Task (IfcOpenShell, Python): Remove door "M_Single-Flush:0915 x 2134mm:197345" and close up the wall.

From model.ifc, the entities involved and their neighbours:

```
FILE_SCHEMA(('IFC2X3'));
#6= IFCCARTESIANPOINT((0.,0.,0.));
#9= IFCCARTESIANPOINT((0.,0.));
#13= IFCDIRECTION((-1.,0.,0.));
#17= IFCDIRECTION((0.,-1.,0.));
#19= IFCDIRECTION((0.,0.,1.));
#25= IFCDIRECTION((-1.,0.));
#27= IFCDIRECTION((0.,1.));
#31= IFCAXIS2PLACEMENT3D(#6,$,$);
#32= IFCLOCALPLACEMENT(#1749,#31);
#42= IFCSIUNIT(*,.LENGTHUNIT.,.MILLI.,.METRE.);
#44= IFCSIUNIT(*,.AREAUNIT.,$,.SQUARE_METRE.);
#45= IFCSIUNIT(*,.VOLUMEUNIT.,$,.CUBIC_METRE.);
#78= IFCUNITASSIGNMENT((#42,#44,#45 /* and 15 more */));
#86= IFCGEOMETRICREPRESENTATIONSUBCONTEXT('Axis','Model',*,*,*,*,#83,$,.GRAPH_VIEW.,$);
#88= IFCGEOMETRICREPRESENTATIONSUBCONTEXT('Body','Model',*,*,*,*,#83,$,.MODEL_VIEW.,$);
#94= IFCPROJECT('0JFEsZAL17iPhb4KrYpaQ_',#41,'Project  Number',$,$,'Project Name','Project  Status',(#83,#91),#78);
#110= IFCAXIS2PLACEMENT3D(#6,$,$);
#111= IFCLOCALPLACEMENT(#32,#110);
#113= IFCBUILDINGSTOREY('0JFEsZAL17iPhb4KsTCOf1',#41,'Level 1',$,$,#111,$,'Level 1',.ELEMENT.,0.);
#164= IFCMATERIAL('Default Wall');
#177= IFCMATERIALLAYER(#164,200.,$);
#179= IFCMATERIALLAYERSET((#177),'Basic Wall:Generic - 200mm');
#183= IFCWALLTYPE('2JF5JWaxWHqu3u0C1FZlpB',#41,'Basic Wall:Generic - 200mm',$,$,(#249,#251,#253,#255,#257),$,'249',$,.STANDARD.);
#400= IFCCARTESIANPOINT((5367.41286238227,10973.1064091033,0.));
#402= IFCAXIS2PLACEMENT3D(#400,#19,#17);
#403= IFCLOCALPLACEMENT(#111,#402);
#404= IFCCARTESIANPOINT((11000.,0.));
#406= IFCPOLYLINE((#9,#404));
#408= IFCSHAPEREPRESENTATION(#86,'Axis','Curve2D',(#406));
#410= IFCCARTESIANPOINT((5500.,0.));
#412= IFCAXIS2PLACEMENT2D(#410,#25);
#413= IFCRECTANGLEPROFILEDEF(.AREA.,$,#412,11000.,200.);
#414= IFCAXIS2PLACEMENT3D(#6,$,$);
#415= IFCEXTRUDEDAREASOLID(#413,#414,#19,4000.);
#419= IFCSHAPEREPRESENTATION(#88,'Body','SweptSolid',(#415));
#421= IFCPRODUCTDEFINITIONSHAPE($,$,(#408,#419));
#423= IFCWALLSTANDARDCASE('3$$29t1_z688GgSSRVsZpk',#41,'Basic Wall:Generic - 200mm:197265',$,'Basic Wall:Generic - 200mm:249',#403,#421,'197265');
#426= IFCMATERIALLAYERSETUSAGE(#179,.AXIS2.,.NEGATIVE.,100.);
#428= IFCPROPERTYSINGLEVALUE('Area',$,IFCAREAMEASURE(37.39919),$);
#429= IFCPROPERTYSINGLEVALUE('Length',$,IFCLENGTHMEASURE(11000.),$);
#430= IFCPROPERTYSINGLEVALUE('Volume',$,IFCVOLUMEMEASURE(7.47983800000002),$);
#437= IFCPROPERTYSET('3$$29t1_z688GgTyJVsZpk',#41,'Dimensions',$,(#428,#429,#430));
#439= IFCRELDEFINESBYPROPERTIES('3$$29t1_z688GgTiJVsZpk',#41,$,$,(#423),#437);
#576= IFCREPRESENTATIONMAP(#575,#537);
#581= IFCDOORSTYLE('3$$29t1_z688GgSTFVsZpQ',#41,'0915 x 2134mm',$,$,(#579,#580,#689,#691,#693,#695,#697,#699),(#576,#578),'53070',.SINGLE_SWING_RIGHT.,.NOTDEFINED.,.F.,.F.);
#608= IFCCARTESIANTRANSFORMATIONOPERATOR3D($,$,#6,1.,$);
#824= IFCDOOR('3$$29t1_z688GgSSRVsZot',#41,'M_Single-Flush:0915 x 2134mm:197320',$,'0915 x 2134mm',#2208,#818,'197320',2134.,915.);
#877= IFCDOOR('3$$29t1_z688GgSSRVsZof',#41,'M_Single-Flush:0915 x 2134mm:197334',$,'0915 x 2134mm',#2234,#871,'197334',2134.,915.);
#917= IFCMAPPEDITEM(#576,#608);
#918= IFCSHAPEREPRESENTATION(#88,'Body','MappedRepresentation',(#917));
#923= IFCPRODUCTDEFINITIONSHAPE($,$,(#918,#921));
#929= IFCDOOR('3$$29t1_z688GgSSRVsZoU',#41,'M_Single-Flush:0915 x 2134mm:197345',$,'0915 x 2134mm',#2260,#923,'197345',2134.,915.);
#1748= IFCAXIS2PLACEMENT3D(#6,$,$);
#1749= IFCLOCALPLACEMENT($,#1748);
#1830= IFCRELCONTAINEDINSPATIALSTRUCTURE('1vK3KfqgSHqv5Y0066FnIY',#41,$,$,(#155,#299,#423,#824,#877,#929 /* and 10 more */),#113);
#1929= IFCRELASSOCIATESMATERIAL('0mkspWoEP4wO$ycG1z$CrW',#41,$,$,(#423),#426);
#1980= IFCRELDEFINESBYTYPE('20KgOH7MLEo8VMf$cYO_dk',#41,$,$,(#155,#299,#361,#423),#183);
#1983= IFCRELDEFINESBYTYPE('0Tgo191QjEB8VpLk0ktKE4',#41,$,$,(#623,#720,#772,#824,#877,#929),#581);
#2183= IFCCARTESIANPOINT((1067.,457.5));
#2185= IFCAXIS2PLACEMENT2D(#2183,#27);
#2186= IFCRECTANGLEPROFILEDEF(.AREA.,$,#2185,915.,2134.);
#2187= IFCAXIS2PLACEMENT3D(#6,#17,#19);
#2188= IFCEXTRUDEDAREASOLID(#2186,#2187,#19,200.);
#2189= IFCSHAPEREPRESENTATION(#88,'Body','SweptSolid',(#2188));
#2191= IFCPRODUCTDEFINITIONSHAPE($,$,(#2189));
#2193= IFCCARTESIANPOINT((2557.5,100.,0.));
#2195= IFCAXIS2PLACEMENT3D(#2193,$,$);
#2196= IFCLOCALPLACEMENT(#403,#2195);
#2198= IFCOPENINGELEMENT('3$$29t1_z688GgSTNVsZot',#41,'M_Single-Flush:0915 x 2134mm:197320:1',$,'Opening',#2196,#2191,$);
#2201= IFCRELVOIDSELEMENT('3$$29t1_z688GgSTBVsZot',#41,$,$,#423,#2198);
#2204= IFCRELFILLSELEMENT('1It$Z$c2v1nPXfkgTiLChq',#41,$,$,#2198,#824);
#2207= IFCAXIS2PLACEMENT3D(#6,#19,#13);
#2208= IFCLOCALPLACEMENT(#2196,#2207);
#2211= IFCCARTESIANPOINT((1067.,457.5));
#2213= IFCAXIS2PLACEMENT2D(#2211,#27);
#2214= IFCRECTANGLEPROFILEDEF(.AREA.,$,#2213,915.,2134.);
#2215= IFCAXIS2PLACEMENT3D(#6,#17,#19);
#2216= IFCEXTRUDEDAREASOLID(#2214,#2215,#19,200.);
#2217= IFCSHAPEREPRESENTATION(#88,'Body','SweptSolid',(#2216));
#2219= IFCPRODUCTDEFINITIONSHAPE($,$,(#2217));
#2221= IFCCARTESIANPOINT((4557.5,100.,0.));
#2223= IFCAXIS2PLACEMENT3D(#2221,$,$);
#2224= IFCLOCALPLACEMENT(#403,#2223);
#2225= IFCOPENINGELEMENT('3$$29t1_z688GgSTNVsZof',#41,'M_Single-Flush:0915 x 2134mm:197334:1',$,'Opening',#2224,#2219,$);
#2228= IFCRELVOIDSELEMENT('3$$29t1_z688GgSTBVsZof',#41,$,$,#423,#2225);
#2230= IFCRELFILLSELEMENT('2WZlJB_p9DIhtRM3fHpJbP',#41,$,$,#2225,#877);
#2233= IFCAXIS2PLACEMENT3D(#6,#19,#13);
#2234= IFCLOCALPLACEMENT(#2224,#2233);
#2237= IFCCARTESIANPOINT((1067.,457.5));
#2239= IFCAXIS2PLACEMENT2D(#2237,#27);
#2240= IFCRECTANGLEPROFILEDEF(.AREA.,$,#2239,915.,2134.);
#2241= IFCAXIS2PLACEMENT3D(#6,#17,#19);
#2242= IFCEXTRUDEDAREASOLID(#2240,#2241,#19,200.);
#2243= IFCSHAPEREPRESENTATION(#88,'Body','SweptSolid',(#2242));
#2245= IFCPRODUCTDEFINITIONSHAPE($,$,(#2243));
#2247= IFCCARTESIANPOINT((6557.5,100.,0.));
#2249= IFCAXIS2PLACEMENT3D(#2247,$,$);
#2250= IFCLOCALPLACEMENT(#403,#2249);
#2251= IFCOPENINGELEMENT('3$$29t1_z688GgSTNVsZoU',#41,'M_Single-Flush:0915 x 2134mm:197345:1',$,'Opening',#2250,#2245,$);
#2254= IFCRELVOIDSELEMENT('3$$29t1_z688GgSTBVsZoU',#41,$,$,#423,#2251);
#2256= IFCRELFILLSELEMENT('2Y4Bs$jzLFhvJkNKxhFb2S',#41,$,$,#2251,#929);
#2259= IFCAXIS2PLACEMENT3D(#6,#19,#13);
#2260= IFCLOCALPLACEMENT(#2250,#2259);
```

```python
import ifcopenshell
import ifcopenshell.api.feature
import ifcopenshell.api.pset
import ifcopenshell.api.root
import ifcopenshell.geom
import ifcopenshell.util.element
import ifcopenshell.util.shape
import ifcopenshell.util.unit

model = ifcopenshell.open("model.ifc")
area_scale = ifcopenshell.util.unit.calculate_unit_scale(model, "AREAUNIT")
volume_scale = ifcopenshell.util.unit.calculate_unit_scale(model, "VOLUMEUNIT")
settings = ifcopenshell.geom.settings()


def volume(element):
    """Net volume in cubic metres, openings subtracted."""
    shape = ifcopenshell.geom.create_shape(settings, element)
    return ifcopenshell.util.shape.get_volume(shape.geometry)


door = model.by_id(929)
opening = door.FillsVoids[0].RelatingOpeningElement
wall = opening.VoidsElements[0].RelatingBuildingElement
before = volume(wall)

ifcopenshell.api.root.remove_product(model, product=door)
ifcopenshell.api.feature.remove_feature(model, feature=opening)

after = volume(wall)
thickness = 0.2  # wall thickness in metres

# Update the wall's stored quantities.
pset = model.by_id(ifcopenshell.util.element.get_pset(wall, "Dimensions", should_inherit=False)["id"])
ifcopenshell.api.pset.edit_pset(model, pset=pset, properties={
    "Area": model.create_entity("IfcAreaMeasure", after / thickness / area_scale),
    "Volume": model.create_entity("IfcVolumeMeasure", after / volume_scale),
})

print(f"wall volume {before:.3f} -> {after:.3f} m3")

model.write("model_updated.ifc")
```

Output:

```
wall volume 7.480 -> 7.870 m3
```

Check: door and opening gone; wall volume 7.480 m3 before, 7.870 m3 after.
